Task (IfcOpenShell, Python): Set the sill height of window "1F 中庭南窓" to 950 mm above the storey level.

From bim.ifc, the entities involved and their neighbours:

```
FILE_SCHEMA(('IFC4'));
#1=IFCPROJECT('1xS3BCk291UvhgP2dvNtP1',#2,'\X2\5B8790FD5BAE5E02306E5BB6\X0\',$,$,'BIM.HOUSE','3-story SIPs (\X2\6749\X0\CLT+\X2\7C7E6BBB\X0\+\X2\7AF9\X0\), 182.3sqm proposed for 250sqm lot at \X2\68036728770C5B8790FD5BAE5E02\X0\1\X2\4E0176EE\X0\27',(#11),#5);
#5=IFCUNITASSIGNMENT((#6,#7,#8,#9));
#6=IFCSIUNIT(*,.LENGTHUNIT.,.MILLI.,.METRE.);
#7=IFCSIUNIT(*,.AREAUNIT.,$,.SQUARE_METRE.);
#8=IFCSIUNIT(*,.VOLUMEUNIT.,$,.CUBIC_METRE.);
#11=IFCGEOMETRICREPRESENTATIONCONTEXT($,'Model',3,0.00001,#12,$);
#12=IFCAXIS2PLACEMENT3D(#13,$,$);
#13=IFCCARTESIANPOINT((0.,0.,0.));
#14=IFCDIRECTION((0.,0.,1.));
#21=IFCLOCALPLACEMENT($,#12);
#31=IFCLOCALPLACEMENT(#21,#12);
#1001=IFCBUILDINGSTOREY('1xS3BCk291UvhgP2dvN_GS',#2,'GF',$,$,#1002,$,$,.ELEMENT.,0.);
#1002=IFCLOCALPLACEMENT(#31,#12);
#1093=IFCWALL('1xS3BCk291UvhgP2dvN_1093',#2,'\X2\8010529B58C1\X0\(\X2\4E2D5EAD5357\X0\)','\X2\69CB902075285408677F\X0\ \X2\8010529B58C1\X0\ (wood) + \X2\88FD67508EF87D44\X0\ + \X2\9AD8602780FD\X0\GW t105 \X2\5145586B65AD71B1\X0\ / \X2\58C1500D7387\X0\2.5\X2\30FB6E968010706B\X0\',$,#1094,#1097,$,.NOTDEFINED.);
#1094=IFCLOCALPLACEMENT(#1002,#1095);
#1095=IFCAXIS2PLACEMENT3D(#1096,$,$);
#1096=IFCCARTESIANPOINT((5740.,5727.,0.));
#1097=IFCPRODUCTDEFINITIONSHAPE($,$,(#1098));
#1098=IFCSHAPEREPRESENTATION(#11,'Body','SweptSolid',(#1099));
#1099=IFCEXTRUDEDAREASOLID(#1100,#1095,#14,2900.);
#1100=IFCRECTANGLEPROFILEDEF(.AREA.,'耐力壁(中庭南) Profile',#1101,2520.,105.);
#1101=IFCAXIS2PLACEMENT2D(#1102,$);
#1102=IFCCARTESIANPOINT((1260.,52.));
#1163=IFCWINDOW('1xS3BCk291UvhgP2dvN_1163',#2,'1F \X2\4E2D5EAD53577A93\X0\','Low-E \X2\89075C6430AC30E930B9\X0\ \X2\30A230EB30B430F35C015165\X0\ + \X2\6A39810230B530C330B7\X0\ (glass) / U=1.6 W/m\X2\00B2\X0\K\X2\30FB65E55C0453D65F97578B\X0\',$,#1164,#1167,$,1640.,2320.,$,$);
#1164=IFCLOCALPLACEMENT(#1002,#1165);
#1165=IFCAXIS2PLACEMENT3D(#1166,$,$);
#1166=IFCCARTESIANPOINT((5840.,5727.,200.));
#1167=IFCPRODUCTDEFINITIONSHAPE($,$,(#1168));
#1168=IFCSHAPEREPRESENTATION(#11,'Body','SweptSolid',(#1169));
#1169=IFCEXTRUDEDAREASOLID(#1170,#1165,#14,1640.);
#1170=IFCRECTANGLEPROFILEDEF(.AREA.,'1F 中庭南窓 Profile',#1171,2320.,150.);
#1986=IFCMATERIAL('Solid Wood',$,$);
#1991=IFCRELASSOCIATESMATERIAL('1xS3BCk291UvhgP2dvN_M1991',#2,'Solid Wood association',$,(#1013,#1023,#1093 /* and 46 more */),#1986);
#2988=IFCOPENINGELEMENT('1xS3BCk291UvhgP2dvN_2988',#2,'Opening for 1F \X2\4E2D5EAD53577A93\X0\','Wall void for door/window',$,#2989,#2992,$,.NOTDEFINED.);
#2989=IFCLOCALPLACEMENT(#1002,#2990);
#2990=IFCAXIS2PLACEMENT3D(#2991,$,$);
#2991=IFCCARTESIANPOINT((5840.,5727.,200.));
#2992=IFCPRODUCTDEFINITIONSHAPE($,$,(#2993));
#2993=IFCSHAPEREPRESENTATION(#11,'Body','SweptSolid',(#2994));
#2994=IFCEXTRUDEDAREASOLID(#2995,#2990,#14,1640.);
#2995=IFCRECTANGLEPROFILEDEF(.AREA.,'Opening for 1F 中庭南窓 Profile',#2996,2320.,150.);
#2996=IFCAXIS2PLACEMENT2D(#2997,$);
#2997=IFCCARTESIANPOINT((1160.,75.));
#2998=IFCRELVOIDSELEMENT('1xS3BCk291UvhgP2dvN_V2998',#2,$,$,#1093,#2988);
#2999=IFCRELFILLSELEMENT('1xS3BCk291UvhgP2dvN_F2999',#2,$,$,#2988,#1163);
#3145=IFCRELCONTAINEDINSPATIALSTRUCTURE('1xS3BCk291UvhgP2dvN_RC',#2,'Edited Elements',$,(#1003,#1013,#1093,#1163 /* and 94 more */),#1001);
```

```python
import numpy as np
import ifcopenshell
import ifcopenshell.api.geometry
import ifcopenshell.geom
import ifcopenshell.util.element
import ifcopenshell.util.placement
import ifcopenshell.util.shape
import ifcopenshell.util.unit

model = ifcopenshell.open("bim.ifc")
unit_scale = ifcopenshell.util.unit.calculate_unit_scale(model)

window = model.by_guid("1xS3BCk291UvhgP2dvN_1163")
opening = window.FillsVoids[0].RelatingOpeningElement
storey = ifcopenshell.util.element.get_container(window, ifc_class="IfcBuildingStorey")
level = ifcopenshell.util.placement.get_local_placement(storey.ObjectPlacement)[2, 3]

# The opening's origin need not be at the sill, so measure its lowest point.
shape = ifcopenshell.geom.create_shape(ifcopenshell.geom.settings(), opening)
bottom = ifcopenshell.util.shape.get_shape_bottom_elevation(shape, shape.geometry) / unit_scale
dz = level + 0.95 / unit_scale - bottom

shift = np.array([0.0, 0.0, dz])
# The window is not placed relative to its opening, so move both.
for product in (opening, window):
    matrix = ifcopenshell.util.placement.get_local_placement(product.ObjectPlacement)
    matrix[:3, 3] += shift
    ifcopenshell.api.geometry.edit_object_placement(model, product=product, matrix=matrix, is_si=False)

print(f"moved by {dz * unit_scale:+.3f} m")

model.write("bim_v2.ifc")
```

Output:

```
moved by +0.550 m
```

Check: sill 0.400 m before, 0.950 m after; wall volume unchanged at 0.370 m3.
